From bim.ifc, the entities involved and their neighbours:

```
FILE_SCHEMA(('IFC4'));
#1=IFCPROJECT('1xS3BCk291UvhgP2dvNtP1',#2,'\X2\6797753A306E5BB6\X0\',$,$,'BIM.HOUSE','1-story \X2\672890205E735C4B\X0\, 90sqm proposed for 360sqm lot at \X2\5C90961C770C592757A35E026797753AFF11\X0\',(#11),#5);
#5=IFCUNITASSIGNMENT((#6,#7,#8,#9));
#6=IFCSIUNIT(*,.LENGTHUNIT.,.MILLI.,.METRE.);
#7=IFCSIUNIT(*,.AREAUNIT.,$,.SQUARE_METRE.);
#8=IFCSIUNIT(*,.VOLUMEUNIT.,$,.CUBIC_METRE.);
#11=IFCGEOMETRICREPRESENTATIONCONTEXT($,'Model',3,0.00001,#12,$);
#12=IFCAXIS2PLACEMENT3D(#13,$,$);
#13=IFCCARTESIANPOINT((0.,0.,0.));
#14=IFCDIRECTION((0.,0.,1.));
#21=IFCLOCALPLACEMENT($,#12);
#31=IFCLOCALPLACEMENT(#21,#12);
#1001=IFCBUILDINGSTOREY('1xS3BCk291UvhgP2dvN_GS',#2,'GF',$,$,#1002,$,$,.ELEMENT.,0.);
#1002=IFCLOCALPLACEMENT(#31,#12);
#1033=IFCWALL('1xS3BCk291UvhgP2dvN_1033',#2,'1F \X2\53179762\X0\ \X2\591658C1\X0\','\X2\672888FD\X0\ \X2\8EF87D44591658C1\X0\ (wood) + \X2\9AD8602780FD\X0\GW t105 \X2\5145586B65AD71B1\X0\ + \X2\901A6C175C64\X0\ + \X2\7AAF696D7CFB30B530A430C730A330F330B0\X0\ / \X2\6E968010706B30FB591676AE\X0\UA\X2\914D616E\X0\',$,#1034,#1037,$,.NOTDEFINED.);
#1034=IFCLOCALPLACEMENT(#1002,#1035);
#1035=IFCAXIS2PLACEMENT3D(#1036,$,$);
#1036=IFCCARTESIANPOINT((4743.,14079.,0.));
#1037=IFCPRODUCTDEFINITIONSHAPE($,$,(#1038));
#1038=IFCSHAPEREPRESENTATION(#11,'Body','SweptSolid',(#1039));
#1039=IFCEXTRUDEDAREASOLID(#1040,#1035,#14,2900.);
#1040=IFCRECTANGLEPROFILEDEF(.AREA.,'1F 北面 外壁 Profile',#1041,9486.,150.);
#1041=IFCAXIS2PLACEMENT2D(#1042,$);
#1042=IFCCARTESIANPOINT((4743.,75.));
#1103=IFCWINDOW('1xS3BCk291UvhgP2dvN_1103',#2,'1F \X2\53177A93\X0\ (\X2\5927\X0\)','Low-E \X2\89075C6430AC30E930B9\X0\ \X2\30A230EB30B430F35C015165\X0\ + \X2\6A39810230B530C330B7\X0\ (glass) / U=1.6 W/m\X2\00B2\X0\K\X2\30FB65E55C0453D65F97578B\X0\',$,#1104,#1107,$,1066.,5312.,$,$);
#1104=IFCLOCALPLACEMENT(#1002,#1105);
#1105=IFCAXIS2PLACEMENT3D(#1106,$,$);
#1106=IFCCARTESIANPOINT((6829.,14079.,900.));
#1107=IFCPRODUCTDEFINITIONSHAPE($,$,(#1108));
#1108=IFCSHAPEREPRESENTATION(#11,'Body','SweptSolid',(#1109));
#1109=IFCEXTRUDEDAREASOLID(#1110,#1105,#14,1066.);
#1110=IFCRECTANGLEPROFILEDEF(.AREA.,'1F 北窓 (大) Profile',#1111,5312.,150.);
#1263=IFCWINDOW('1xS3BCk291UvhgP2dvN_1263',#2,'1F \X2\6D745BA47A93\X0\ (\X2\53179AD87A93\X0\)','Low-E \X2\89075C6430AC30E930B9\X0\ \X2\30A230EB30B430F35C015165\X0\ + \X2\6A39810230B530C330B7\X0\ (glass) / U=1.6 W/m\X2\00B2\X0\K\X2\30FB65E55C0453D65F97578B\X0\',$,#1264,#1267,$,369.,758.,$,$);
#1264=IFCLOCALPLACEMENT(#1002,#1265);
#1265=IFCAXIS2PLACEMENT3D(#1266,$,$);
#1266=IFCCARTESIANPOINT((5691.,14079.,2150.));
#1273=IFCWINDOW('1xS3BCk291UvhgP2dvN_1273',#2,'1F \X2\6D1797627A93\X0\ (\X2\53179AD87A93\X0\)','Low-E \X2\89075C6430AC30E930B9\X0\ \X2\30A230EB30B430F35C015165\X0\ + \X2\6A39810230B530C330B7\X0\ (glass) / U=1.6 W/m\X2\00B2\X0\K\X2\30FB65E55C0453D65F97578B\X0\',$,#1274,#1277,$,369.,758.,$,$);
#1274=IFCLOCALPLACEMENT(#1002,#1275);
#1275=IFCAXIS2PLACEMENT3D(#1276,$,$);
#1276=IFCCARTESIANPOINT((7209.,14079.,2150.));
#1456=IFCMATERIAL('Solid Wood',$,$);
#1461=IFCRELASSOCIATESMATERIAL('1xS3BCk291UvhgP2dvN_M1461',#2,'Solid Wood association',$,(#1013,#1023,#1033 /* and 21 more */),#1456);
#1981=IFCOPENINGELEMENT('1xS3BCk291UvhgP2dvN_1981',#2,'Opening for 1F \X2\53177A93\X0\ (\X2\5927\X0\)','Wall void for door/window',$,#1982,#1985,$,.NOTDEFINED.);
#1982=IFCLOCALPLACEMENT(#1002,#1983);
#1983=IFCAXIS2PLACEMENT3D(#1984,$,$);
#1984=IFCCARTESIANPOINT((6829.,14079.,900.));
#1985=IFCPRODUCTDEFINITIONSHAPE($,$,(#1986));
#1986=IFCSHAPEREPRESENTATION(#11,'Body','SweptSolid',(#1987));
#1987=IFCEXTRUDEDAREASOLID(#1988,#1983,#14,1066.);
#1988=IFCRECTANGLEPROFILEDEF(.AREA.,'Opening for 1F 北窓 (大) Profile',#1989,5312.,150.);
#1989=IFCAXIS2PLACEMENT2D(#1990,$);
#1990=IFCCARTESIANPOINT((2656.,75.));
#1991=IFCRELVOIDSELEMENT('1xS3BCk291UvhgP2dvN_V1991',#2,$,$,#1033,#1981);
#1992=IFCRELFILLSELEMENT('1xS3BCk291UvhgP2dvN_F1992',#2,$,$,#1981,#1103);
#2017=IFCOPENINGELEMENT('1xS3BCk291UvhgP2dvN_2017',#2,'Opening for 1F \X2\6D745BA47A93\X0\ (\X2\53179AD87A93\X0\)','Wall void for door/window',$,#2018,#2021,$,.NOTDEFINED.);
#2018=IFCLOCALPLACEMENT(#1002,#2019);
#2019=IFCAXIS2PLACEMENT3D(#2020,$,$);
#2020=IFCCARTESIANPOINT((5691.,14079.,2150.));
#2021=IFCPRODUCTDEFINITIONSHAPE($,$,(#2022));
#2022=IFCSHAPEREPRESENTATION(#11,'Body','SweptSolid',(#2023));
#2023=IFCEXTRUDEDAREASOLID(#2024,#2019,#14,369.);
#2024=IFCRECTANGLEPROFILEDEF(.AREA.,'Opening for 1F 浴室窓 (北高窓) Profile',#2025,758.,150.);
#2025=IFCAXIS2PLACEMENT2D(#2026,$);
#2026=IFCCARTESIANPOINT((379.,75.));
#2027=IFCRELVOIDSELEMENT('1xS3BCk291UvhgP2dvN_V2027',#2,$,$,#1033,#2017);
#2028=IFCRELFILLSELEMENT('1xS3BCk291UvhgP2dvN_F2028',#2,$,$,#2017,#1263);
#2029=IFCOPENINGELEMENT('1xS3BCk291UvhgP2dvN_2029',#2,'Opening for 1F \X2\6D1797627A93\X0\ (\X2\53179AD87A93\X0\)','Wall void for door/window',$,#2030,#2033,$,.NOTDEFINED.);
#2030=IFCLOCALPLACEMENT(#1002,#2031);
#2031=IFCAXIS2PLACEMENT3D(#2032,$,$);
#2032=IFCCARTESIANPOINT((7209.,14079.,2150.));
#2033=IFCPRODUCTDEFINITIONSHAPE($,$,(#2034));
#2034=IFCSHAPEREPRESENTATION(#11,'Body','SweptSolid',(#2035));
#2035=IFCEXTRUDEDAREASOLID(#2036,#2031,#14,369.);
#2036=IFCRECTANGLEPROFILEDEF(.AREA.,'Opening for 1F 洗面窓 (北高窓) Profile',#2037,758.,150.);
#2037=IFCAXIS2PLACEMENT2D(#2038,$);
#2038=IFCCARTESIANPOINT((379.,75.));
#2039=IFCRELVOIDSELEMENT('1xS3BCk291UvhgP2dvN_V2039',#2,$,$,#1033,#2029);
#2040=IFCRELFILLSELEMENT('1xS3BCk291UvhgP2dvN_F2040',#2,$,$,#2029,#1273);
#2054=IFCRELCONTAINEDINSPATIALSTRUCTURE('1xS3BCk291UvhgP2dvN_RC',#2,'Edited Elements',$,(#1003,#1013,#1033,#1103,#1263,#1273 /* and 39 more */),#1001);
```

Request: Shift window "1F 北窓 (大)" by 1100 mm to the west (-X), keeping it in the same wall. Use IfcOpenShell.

```python
import ifcopenshell
import ifcopenshell.api.geometry
import ifcopenshell.util.placement

model = ifcopenshell.open("bim.ifc")

window = model.by_guid("1xS3BCk291UvhgP2dvN_1103")
opening = window.FillsVoids[0].RelatingOpeningElement
wall = opening.VoidsElements[0].RelatingBuildingElement

wall_matrix = ifcopenshell.util.placement.get_local_placement(wall.ObjectPlacement)
shift = wall_matrix[:3, 0] * -1100.0
before = ifcopenshell.util.placement.get_local_placement(window.ObjectPlacement)[:3, 3].copy()

# The window is not placed relative to its opening, so move both.
for product in (opening, window):
    matrix = ifcopenshell.util.placement.get_local_placement(product.ObjectPlacement)
    matrix[:3, 3] += shift
    ifcopenshell.api.geometry.edit_object_placement(model, product=product, matrix=matrix, is_si=False)

after = ifcopenshell.util.placement.get_local_placement(window.ObjectPlacement)[:3, 3]
print("window moved by", (after - before).round(3) + 0.0)

model.write("bim-out.ifc")
```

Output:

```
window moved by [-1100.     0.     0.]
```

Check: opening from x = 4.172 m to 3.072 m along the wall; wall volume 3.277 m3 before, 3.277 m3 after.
